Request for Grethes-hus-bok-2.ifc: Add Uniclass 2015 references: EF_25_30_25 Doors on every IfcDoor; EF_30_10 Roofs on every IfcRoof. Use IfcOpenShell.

First a look at what the model holds.

```python
import ifcopenshell

model = ifcopenshell.open("Grethes-hus-bok-2.ifc")
print(model.schema)
print("classifications:", [c.Name for c in model.by_type("IfcClassification")])
for ifc_class in ("IfcDoor", "IfcRoof", "IfcStair", "IfcWall", "IfcWindow"):
    print(ifc_class, len(model.by_type(ifc_class)))
```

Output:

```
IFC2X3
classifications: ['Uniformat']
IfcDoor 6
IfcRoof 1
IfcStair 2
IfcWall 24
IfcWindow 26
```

```python
import ifcopenshell
import ifcopenshell.api.classification

model = ifcopenshell.open("Grethes-hus-bok-2.ifc")

# IFC2X3 requires Source and Edition and has no link from the project to the system.
system = model.create_entity("IfcClassification", Source="NBS", Edition="2015", Name="Uniclass 2015")

codes = {
    "IfcDoor": ("EF_25_30_25", "Doors"),
    "IfcRoof": ("EF_30_10", "Roofs"),
}
for ifc_class, (code, name) in codes.items():
    products = model.by_type(ifc_class)
    ifcopenshell.api.classification.add_reference(
        model, products=products, classification=system, identification=code, name=name
    )
    print(code, len(products))

model.write("Grethes-hus-bok-2_edited.ifc")
```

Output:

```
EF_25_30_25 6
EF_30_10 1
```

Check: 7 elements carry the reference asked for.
